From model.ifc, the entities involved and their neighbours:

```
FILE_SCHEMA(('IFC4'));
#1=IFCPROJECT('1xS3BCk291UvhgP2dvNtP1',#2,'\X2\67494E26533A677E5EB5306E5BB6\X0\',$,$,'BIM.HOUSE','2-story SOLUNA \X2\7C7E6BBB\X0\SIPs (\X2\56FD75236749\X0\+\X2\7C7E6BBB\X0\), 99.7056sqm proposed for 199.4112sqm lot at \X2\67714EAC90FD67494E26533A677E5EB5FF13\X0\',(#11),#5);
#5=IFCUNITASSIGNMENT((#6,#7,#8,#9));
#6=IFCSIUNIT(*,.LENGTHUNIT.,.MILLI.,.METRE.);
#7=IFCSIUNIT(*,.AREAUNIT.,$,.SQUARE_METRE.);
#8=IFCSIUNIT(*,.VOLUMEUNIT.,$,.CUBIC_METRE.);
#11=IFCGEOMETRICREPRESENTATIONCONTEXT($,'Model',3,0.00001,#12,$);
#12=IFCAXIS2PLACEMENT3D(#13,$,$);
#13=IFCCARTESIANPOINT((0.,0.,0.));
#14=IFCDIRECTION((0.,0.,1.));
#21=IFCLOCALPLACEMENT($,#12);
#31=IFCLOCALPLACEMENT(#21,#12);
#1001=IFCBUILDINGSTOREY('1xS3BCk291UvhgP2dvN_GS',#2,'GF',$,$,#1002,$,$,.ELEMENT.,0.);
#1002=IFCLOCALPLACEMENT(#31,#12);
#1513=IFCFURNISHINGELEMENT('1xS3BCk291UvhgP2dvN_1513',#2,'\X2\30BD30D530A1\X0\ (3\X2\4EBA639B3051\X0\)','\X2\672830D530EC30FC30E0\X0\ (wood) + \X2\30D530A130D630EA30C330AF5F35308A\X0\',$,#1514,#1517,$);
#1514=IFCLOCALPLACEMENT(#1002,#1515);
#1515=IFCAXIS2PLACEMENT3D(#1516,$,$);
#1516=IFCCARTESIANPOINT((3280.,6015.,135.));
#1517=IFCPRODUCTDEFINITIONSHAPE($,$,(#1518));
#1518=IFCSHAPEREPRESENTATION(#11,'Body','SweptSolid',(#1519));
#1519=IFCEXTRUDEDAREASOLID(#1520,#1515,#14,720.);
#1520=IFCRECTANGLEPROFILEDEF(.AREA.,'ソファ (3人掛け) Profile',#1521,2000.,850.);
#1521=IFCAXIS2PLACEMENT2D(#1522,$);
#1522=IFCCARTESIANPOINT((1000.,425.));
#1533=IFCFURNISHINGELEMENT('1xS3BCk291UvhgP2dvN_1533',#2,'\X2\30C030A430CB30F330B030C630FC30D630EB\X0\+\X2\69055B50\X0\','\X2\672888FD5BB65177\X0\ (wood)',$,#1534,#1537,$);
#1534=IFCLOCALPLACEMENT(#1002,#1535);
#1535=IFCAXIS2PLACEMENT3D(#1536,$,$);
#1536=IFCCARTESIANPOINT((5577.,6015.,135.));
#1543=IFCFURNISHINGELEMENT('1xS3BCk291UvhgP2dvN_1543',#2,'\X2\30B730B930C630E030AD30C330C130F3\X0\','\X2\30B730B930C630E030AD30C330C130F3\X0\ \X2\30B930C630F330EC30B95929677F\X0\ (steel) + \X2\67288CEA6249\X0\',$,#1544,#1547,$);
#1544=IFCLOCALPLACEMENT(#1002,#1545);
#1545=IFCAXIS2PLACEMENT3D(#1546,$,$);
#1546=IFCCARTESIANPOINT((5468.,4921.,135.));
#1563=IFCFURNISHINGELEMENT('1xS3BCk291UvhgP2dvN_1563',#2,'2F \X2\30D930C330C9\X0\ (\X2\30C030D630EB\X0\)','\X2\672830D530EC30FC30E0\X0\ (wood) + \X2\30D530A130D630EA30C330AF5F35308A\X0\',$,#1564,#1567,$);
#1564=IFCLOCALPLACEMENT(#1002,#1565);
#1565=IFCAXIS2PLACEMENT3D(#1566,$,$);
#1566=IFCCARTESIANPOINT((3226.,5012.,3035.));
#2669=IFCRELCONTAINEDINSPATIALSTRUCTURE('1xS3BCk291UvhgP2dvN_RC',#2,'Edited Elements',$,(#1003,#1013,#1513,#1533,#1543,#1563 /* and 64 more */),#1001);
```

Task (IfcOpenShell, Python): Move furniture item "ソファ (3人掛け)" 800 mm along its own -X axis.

```python
import ifcopenshell
import ifcopenshell.api.geometry
import ifcopenshell.util.placement

model = ifcopenshell.open("model.ifc")

item = model.by_guid("1xS3BCk291UvhgP2dvN_1513")
matrix = ifcopenshell.util.placement.get_local_placement(item.ObjectPlacement)
matrix[:3, 3] -= matrix[:3, 0] * 800.0
ifcopenshell.api.geometry.edit_object_placement(model, product=item, matrix=matrix, is_si=False)

print(ifcopenshell.util.placement.get_local_placement(item.ObjectPlacement).round(3) + 0.0)

model.write("model_edited.ifc")
```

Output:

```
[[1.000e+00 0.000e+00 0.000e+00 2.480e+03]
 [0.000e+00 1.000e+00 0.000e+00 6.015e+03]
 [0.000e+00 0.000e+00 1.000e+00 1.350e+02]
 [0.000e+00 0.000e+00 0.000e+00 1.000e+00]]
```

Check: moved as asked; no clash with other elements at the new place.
